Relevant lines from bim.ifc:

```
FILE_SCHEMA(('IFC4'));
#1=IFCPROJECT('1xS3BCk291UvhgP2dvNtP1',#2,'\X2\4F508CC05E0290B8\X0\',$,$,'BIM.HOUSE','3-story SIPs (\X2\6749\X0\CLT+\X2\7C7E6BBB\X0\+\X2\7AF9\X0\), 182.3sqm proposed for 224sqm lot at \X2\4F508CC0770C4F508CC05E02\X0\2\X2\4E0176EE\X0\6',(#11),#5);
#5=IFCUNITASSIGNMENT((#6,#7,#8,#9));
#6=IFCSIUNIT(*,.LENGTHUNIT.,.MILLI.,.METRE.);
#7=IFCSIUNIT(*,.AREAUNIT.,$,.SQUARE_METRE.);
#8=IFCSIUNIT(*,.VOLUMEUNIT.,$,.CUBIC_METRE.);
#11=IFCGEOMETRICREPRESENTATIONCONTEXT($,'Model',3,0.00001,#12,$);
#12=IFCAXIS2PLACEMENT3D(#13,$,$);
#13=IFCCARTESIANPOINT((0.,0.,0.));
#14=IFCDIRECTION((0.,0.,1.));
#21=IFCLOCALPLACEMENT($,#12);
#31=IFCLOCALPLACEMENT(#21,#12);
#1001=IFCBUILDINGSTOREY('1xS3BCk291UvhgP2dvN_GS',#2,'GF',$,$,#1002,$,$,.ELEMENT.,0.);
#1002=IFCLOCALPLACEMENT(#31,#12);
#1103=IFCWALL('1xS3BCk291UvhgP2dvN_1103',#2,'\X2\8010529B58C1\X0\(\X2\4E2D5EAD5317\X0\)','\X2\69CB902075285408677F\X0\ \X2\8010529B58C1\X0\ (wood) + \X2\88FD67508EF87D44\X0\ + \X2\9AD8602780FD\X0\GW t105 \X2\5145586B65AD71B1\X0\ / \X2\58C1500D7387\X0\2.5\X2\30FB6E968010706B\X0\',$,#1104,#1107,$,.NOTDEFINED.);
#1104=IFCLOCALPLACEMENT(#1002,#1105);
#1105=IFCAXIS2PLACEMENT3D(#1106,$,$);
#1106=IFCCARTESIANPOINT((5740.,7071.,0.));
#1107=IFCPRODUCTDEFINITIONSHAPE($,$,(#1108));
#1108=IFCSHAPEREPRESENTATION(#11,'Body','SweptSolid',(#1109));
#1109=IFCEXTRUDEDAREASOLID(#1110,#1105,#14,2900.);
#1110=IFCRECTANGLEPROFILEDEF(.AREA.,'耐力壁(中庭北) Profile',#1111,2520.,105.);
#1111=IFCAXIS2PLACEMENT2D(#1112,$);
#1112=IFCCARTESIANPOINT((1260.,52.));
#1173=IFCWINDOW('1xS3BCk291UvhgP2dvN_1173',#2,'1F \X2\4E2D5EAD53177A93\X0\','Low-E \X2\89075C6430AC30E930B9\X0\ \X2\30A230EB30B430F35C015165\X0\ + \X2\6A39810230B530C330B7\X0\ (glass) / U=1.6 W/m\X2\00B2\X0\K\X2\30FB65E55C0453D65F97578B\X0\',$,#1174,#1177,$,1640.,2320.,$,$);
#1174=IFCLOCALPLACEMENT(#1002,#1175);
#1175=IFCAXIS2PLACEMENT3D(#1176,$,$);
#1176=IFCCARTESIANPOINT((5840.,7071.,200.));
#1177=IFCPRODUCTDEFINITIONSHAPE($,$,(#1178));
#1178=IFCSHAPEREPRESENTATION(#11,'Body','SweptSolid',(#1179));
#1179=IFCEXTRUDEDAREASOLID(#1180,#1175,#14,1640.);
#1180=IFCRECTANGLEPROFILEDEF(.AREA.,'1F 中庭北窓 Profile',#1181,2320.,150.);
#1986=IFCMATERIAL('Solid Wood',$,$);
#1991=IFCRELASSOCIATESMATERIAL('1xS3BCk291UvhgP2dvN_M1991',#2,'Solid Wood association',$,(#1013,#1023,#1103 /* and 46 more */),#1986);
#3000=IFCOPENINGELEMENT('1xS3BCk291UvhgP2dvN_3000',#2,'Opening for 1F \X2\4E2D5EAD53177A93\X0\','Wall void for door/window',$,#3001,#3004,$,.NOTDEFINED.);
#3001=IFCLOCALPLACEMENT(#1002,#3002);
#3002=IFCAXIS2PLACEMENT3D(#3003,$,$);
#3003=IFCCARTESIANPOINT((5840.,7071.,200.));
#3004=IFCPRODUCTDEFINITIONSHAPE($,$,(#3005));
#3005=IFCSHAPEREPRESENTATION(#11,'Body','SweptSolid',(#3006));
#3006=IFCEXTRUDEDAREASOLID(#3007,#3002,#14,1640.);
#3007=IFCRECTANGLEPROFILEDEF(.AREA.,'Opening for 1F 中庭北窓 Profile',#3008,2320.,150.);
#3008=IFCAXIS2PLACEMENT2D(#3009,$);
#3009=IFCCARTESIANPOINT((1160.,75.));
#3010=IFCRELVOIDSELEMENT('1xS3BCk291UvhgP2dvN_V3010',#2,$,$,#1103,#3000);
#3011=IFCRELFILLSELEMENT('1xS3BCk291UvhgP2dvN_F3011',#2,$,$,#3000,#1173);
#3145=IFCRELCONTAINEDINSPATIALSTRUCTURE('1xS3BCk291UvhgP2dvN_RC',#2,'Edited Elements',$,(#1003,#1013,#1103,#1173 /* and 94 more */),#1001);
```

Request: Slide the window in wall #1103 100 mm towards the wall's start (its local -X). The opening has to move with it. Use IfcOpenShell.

```python
import ifcopenshell
import ifcopenshell.api.geometry
import ifcopenshell.util.placement
import ifcopenshell.util.unit

model = ifcopenshell.open("bim.ifc")
unit_scale = ifcopenshell.util.unit.calculate_unit_scale(model)

window = model.by_guid("1xS3BCk291UvhgP2dvN_1173")
opening = window.FillsVoids[0].RelatingOpeningElement
wall = opening.VoidsElements[0].RelatingBuildingElement

wall_matrix = ifcopenshell.util.placement.get_local_placement(wall.ObjectPlacement)
shift = wall_matrix[:3, 0] * -0.1 / unit_scale
before = ifcopenshell.util.placement.get_local_placement(window.ObjectPlacement)[:3, 3].copy()

# The window is not placed relative to its opening, so move both.
for product in (opening, window):
    matrix = ifcopenshell.util.placement.get_local_placement(product.ObjectPlacement)
    matrix[:3, 3] += shift
    ifcopenshell.api.geometry.edit_object_placement(model, product=product, matrix=matrix, is_si=False)

after = ifcopenshell.util.placement.get_local_placement(window.ObjectPlacement)[:3, 3]
print("window moved by", (after - before).round(3) + 0.0)

model.write("bim_v2.ifc")
```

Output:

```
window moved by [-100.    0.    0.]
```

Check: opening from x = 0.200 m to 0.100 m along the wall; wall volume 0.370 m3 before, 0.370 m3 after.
